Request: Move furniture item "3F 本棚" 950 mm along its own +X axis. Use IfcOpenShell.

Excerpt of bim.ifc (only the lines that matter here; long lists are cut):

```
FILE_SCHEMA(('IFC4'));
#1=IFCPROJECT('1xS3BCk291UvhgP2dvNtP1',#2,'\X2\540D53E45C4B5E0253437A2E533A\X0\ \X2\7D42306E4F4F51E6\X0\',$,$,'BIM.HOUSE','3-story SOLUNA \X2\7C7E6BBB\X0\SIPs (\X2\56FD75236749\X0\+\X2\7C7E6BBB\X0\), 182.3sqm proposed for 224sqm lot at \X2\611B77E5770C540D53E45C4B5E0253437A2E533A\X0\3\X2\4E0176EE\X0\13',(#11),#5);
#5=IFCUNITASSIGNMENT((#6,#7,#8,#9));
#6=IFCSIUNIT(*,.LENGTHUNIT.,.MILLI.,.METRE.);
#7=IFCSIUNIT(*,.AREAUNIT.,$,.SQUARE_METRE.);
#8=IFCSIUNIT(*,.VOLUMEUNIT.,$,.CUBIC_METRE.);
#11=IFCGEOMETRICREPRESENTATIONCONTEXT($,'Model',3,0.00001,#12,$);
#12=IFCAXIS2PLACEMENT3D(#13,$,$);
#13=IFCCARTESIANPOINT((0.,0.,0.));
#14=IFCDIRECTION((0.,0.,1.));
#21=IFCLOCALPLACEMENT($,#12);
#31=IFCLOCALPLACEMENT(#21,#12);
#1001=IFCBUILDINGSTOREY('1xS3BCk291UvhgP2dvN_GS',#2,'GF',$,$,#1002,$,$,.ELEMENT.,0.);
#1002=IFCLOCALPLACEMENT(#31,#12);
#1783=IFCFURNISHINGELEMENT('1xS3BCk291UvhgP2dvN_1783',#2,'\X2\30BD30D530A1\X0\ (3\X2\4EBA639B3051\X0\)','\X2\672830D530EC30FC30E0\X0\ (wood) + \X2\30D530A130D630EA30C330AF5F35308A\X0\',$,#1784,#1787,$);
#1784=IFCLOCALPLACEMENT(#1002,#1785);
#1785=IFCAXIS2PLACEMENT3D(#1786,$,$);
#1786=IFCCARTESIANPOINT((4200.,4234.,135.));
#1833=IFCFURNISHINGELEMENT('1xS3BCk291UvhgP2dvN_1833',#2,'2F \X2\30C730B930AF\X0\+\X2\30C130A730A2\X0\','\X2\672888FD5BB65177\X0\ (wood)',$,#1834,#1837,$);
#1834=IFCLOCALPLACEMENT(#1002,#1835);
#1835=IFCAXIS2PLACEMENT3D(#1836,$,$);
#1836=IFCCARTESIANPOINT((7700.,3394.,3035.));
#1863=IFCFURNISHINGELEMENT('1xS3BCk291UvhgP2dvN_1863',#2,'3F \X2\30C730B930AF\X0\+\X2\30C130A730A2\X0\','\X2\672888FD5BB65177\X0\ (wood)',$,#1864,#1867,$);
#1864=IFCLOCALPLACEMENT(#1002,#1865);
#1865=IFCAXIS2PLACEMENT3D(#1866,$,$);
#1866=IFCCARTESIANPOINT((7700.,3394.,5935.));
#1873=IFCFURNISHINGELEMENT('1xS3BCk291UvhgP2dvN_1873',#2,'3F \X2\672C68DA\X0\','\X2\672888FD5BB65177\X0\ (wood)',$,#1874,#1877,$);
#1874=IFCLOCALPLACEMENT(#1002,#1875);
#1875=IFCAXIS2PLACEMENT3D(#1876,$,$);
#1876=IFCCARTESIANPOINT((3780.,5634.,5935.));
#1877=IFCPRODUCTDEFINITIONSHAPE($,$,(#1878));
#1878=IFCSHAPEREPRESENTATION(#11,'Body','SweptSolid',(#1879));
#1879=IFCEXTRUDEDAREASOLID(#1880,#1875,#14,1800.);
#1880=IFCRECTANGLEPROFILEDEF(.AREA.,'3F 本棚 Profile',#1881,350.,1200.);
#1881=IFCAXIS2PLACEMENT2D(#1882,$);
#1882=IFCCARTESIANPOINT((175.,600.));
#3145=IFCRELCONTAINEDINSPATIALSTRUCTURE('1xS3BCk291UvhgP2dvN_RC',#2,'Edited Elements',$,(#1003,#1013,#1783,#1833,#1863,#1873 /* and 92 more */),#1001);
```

```python
import ifcopenshell
import ifcopenshell.api.geometry
import ifcopenshell.util.placement

model = ifcopenshell.open("bim.ifc")

item = model.by_guid("1xS3BCk291UvhgP2dvN_1873")
matrix = ifcopenshell.util.placement.get_local_placement(item.ObjectPlacement)
matrix[:3, 3] += matrix[:3, 0] * 950.0
ifcopenshell.api.geometry.edit_object_placement(model, product=item, matrix=matrix, is_si=False)

print(ifcopenshell.util.placement.get_local_placement(item.ObjectPlacement).round(3) + 0.0)

model.write("bim_v2.ifc")
```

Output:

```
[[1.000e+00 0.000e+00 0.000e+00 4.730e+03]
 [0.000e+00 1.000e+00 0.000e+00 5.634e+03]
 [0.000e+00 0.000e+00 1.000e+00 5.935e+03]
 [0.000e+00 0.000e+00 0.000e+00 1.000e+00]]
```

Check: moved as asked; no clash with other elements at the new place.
